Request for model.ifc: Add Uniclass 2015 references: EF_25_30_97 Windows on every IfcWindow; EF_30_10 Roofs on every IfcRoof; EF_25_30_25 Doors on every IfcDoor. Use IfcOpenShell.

First a look at what the model holds.

```python
import ifcopenshell

model = ifcopenshell.open("model.ifc")
print(model.schema)
print("classifications:", [c.Name for c in model.by_type("IfcClassification")])
for ifc_class in ("IfcDoor", "IfcRoof", "IfcStair", "IfcWall", "IfcWindow"):
    print(ifc_class, len(model.by_type(ifc_class)))
```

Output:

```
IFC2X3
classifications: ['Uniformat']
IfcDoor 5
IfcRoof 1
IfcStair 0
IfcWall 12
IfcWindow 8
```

```python
import ifcopenshell
import ifcopenshell.api.classification

model = ifcopenshell.open("model.ifc")

# IFC2X3 requires Source and Edition and has no link from the project to the system.
system = model.create_entity("IfcClassification", Source="NBS", Edition="2015", Name="Uniclass 2015")

codes = {
    "IfcWindow": ("EF_25_30_97", "Windows"),
    "IfcRoof": ("EF_30_10", "Roofs"),
    "IfcDoor": ("EF_25_30_25", "Doors"),
}
for ifc_class, (code, name) in codes.items():
    products = model.by_type(ifc_class)
    ifcopenshell.api.classification.add_reference(
        model, products=products, classification=system, identification=code, name=name
    )
    print(code, len(products))

model.write("model_edited.ifc")
```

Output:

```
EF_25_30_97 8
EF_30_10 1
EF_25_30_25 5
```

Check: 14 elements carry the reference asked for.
